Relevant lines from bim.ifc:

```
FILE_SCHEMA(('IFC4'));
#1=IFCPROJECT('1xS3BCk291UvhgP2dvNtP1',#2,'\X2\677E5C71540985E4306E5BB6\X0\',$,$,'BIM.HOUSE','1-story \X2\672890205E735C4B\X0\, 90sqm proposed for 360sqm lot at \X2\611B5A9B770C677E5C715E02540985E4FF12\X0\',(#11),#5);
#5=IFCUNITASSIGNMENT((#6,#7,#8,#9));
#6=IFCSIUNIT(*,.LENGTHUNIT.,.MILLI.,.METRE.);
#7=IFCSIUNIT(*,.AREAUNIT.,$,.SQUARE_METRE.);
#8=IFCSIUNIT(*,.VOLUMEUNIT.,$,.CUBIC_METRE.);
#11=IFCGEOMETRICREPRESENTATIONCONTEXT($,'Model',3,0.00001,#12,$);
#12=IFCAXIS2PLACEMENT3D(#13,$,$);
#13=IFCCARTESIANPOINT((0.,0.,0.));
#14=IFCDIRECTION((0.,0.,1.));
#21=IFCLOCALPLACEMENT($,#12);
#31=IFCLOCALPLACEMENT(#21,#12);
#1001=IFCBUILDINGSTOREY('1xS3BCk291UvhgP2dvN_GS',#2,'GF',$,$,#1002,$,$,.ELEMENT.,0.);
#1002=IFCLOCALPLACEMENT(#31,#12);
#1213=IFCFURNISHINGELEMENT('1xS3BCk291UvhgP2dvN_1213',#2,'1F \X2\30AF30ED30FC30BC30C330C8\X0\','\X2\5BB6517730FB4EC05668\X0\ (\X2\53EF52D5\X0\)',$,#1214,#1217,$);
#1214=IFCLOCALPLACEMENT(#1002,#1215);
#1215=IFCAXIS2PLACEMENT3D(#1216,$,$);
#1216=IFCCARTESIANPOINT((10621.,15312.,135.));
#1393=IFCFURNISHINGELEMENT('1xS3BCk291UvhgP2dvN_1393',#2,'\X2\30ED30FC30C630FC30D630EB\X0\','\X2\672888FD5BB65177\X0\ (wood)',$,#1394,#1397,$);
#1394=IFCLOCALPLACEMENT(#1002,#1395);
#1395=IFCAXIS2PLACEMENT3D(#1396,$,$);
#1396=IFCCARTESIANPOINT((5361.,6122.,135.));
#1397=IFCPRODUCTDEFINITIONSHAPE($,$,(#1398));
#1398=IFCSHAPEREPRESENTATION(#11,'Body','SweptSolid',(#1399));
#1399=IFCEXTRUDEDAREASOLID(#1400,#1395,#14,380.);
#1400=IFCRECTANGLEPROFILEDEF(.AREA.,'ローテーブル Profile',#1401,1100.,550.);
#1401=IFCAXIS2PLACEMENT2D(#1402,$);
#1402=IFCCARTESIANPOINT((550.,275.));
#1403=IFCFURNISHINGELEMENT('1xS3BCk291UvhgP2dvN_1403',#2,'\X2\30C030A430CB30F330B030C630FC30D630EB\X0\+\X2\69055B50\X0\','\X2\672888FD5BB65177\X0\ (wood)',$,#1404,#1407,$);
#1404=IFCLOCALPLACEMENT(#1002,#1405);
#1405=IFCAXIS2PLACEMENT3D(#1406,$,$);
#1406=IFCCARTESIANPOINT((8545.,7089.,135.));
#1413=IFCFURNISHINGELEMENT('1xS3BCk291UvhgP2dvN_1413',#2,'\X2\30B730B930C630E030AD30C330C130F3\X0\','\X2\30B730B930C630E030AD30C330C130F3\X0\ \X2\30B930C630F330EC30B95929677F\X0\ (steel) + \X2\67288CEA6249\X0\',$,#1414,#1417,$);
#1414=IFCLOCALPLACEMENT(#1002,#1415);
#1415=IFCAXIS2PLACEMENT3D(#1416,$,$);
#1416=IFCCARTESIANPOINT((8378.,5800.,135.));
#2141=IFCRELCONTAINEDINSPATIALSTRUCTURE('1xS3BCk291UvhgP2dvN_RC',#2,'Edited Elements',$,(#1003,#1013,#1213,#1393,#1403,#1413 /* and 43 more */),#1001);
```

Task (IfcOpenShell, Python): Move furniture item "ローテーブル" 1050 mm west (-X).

```python
import ifcopenshell
import ifcopenshell.api.geometry
import ifcopenshell.util.placement
import ifcopenshell.util.unit

model = ifcopenshell.open("bim.ifc")
unit_scale = ifcopenshell.util.unit.calculate_unit_scale(model)

item = model.by_guid("1xS3BCk291UvhgP2dvN_1393")
matrix = ifcopenshell.util.placement.get_local_placement(item.ObjectPlacement)
matrix[0, 3] -= 1.05 / unit_scale
ifcopenshell.api.geometry.edit_object_placement(model, product=item, matrix=matrix, is_si=False)

print(ifcopenshell.util.placement.get_local_placement(item.ObjectPlacement).round(3) + 0.0)

model.write("bim_v2.ifc")
```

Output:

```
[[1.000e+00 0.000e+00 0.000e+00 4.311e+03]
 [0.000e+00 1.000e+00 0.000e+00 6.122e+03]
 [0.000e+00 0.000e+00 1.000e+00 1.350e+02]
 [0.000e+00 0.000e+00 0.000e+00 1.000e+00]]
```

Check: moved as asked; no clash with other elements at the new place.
